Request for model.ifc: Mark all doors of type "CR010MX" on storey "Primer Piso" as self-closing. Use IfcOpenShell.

First a look at what the model holds.

```python
import ifcopenshell
import ifcopenshell.util.element

model = ifcopenshell.open("model.ifc")
print(model.schema)
storey = next(s for s in model.by_type("IfcBuildingStorey") if s.Name == "Primer Piso")
doors = [e for e in ifcopenshell.util.element.get_decomposition(storey) if e.is_a("IfcDoor")]
seen = {}
for e in doors:
    element_type = ifcopenshell.util.element.get_type(e)
    key = (element_type.Name if element_type != e and element_type else None, ifcopenshell.util.element.get_pset(e, "Pset_DoorCommon", "SelfClosing"))
    seen[key] = seen.get(key, 0) + 1
for (name, value), count in sorted(seen.items(), key=str):
    print(count, "x", name, "|", value)
```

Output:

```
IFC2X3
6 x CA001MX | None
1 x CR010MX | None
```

```python
import ifcopenshell
import ifcopenshell.api.pset
import ifcopenshell.util.element

model = ifcopenshell.open("model.ifc")

storey = next(s for s in model.by_type("IfcBuildingStorey") if s.Name == "Primer Piso")
doors = [e for e in ifcopenshell.util.element.get_decomposition(storey) if e.is_a("IfcDoor")]

count = 0
for e in doors:
    element_type = ifcopenshell.util.element.get_type(e)
    if element_type in (None, e) or element_type.Name != "CR010MX":
        continue
    # add_pset returns the element's existing set when there is one.
    pset = ifcopenshell.api.pset.add_pset(model, product=e, name="Pset_DoorCommon")
    ifcopenshell.api.pset.edit_pset(model, pset=pset, properties={"SelfClosing": True})
    count += 1

print(count, "doors updated")

model.write("model_rev.ifc")
```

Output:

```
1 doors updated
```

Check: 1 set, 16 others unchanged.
